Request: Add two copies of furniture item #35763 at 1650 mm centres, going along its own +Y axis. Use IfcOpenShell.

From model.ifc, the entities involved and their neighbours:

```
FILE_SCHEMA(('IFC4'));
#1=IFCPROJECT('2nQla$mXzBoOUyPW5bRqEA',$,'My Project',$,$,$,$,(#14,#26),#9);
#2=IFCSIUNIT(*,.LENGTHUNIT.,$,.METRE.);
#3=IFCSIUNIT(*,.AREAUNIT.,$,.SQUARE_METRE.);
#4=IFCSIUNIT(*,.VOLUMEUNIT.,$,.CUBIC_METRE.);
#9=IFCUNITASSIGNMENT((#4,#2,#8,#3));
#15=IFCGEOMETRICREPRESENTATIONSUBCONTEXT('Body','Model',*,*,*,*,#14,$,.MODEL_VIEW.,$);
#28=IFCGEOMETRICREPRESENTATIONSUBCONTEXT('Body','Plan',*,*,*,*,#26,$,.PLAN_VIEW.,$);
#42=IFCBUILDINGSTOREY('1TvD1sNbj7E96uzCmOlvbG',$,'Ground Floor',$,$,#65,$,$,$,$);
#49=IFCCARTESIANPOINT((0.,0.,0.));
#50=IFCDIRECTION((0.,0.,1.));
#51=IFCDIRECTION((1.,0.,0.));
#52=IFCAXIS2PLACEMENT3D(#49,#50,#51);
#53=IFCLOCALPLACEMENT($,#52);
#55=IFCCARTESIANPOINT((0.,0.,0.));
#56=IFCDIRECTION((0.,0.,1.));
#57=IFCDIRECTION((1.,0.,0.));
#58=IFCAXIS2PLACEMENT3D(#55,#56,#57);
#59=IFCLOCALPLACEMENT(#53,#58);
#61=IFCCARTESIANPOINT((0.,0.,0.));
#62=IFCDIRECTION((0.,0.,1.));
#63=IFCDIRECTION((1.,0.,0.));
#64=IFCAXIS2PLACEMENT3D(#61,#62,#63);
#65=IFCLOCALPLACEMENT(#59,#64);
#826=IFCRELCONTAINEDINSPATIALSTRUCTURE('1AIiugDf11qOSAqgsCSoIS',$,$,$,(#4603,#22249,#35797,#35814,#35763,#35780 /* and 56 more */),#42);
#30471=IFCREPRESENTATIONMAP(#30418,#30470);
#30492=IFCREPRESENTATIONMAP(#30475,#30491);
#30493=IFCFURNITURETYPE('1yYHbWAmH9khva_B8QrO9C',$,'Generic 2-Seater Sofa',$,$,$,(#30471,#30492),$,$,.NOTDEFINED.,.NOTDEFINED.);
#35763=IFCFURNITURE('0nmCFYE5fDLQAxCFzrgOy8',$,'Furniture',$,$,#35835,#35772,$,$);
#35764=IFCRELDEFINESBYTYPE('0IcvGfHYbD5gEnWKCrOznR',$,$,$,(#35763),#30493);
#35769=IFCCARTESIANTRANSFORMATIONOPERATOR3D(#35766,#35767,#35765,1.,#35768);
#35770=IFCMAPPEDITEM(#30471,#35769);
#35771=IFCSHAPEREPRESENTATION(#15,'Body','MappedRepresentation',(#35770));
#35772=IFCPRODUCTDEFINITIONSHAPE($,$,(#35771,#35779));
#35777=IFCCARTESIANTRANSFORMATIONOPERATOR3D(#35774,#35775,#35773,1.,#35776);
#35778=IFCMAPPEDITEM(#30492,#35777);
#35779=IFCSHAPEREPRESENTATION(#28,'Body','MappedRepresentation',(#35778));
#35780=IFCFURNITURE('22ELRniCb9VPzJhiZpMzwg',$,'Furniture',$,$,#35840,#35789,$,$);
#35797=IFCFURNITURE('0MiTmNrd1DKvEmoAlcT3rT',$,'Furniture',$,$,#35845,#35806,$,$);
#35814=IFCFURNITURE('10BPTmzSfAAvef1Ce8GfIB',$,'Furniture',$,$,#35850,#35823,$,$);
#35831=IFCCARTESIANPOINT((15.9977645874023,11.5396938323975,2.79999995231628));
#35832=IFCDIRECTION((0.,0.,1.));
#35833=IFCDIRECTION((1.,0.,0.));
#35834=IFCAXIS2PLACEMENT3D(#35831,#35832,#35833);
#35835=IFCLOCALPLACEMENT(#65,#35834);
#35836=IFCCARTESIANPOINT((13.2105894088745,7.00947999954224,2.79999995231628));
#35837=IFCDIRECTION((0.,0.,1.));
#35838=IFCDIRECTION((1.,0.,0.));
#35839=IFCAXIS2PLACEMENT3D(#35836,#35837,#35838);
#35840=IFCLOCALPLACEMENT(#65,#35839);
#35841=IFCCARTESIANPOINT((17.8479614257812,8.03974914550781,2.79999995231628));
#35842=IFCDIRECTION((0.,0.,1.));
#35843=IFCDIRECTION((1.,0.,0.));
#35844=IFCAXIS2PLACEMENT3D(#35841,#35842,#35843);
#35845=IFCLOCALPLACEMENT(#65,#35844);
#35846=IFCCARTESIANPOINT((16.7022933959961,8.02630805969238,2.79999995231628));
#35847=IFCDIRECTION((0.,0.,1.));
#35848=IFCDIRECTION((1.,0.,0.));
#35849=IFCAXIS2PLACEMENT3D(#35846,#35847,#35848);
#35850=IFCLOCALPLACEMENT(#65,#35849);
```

```python
import ifcopenshell
import ifcopenshell.api.geometry
import ifcopenshell.api.root
import ifcopenshell.util.element
import ifcopenshell.util.placement

model = ifcopenshell.open("model.ifc")

source = model.by_guid("0nmCFYE5fDLQAxCFzrgOy8")
base = ifcopenshell.util.placement.get_local_placement(source.ObjectPlacement)
step = base[:3, 1] * 1.65

for i in range(1, 3):
    copy = ifcopenshell.api.root.copy_class(model, product=source)
    copy.Representation = ifcopenshell.util.element.copy_deep(
        model, source.Representation, exclude=["IfcGeometricRepresentationContext", "IfcRepresentationMap"]
    )
    matrix = base.copy()
    matrix[:3, 3] += i * step
    print("added at", matrix[:3, 3].round(3) + 0.0)
    ifcopenshell.api.geometry.edit_object_placement(model, product=copy, matrix=matrix, is_si=False)

model.write("model_edited.ifc")
```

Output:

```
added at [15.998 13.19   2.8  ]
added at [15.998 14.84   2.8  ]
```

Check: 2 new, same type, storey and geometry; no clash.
